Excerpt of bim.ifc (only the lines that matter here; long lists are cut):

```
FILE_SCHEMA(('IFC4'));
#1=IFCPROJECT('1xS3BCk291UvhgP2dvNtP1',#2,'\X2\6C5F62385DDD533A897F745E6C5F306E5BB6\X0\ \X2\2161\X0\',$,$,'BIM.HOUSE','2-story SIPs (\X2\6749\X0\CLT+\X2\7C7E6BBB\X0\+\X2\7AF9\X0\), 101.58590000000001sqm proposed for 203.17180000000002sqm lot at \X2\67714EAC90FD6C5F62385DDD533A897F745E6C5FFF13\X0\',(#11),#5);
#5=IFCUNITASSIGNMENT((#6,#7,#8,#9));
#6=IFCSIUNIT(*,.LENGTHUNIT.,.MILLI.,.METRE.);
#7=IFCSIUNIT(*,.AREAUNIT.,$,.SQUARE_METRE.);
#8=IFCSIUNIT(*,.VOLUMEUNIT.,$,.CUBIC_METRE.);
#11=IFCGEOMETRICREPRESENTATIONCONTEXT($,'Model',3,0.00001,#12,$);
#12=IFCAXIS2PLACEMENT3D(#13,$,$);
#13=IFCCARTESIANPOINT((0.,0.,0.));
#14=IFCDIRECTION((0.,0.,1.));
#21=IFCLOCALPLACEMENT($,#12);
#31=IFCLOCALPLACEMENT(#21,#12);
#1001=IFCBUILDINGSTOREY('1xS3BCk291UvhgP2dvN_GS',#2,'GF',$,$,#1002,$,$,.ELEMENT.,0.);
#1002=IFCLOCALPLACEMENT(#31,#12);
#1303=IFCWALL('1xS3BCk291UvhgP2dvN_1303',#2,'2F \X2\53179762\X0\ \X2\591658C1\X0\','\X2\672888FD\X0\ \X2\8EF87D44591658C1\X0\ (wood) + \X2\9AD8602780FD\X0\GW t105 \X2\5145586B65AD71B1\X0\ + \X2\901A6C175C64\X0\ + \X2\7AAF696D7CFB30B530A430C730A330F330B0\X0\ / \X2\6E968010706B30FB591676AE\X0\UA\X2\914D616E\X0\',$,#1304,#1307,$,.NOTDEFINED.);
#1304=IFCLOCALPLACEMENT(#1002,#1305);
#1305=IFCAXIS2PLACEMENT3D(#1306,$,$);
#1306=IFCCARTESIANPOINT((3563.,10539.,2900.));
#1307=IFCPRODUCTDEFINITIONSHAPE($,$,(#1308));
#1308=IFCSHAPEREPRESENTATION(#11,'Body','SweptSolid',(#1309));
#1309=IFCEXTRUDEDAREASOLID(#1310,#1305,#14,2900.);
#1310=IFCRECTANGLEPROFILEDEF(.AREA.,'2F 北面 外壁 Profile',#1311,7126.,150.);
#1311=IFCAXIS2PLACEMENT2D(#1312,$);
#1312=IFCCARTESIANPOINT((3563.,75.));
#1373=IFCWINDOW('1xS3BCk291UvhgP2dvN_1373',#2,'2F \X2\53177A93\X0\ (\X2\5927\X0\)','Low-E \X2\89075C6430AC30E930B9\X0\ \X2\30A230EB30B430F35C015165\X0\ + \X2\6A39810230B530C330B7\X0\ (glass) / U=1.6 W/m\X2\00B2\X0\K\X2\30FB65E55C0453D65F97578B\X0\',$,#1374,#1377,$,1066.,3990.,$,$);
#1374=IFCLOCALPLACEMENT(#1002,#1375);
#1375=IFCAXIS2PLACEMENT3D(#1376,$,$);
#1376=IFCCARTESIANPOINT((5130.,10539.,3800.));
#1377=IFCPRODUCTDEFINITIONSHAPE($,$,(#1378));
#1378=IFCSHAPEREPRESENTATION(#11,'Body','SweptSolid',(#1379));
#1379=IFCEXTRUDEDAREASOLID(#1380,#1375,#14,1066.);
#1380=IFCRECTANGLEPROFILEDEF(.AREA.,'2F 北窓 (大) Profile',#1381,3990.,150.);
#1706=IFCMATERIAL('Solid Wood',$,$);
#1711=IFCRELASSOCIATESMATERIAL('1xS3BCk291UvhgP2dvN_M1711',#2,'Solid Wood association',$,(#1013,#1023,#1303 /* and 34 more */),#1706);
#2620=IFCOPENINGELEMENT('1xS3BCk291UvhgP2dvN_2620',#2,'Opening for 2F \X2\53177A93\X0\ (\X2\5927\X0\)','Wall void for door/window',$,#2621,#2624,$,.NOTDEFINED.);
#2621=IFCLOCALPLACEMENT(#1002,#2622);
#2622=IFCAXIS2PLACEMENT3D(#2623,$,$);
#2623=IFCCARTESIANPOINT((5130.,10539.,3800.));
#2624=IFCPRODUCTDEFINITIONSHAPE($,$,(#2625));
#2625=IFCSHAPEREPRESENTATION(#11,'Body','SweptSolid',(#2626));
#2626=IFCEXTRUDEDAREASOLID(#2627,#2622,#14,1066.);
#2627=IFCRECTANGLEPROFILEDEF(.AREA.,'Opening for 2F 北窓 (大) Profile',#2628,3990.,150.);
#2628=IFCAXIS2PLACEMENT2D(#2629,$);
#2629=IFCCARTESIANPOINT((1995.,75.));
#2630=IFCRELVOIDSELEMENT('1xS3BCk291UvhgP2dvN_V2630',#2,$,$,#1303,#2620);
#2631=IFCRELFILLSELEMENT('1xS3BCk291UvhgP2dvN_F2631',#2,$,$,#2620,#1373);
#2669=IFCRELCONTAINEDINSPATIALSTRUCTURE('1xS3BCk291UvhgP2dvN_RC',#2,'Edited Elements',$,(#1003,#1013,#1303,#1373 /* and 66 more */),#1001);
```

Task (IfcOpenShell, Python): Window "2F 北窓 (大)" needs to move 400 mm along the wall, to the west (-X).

```python
import ifcopenshell
import ifcopenshell.api.geometry
import ifcopenshell.util.placement
import ifcopenshell.util.unit

model = ifcopenshell.open("bim.ifc")
unit_scale = ifcopenshell.util.unit.calculate_unit_scale(model)

window = model.by_guid("1xS3BCk291UvhgP2dvN_1373")
opening = window.FillsVoids[0].RelatingOpeningElement
wall = opening.VoidsElements[0].RelatingBuildingElement

wall_matrix = ifcopenshell.util.placement.get_local_placement(wall.ObjectPlacement)
shift = wall_matrix[:3, 0] * -0.4 / unit_scale
before = ifcopenshell.util.placement.get_local_placement(window.ObjectPlacement)[:3, 3].copy()

# The window is not placed relative to its opening, so move both.
for product in (opening, window):
    matrix = ifcopenshell.util.placement.get_local_placement(product.ObjectPlacement)
    matrix[:3, 3] += shift
    ifcopenshell.api.geometry.edit_object_placement(model, product=product, matrix=matrix, is_si=False)

after = ifcopenshell.util.placement.get_local_placement(window.ObjectPlacement)[:3, 3]
print("window moved by", (after - before).round(3) + 0.0)

model.write("bim-out.ifc")
```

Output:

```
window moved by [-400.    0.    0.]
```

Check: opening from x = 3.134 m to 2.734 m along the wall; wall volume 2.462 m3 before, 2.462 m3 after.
